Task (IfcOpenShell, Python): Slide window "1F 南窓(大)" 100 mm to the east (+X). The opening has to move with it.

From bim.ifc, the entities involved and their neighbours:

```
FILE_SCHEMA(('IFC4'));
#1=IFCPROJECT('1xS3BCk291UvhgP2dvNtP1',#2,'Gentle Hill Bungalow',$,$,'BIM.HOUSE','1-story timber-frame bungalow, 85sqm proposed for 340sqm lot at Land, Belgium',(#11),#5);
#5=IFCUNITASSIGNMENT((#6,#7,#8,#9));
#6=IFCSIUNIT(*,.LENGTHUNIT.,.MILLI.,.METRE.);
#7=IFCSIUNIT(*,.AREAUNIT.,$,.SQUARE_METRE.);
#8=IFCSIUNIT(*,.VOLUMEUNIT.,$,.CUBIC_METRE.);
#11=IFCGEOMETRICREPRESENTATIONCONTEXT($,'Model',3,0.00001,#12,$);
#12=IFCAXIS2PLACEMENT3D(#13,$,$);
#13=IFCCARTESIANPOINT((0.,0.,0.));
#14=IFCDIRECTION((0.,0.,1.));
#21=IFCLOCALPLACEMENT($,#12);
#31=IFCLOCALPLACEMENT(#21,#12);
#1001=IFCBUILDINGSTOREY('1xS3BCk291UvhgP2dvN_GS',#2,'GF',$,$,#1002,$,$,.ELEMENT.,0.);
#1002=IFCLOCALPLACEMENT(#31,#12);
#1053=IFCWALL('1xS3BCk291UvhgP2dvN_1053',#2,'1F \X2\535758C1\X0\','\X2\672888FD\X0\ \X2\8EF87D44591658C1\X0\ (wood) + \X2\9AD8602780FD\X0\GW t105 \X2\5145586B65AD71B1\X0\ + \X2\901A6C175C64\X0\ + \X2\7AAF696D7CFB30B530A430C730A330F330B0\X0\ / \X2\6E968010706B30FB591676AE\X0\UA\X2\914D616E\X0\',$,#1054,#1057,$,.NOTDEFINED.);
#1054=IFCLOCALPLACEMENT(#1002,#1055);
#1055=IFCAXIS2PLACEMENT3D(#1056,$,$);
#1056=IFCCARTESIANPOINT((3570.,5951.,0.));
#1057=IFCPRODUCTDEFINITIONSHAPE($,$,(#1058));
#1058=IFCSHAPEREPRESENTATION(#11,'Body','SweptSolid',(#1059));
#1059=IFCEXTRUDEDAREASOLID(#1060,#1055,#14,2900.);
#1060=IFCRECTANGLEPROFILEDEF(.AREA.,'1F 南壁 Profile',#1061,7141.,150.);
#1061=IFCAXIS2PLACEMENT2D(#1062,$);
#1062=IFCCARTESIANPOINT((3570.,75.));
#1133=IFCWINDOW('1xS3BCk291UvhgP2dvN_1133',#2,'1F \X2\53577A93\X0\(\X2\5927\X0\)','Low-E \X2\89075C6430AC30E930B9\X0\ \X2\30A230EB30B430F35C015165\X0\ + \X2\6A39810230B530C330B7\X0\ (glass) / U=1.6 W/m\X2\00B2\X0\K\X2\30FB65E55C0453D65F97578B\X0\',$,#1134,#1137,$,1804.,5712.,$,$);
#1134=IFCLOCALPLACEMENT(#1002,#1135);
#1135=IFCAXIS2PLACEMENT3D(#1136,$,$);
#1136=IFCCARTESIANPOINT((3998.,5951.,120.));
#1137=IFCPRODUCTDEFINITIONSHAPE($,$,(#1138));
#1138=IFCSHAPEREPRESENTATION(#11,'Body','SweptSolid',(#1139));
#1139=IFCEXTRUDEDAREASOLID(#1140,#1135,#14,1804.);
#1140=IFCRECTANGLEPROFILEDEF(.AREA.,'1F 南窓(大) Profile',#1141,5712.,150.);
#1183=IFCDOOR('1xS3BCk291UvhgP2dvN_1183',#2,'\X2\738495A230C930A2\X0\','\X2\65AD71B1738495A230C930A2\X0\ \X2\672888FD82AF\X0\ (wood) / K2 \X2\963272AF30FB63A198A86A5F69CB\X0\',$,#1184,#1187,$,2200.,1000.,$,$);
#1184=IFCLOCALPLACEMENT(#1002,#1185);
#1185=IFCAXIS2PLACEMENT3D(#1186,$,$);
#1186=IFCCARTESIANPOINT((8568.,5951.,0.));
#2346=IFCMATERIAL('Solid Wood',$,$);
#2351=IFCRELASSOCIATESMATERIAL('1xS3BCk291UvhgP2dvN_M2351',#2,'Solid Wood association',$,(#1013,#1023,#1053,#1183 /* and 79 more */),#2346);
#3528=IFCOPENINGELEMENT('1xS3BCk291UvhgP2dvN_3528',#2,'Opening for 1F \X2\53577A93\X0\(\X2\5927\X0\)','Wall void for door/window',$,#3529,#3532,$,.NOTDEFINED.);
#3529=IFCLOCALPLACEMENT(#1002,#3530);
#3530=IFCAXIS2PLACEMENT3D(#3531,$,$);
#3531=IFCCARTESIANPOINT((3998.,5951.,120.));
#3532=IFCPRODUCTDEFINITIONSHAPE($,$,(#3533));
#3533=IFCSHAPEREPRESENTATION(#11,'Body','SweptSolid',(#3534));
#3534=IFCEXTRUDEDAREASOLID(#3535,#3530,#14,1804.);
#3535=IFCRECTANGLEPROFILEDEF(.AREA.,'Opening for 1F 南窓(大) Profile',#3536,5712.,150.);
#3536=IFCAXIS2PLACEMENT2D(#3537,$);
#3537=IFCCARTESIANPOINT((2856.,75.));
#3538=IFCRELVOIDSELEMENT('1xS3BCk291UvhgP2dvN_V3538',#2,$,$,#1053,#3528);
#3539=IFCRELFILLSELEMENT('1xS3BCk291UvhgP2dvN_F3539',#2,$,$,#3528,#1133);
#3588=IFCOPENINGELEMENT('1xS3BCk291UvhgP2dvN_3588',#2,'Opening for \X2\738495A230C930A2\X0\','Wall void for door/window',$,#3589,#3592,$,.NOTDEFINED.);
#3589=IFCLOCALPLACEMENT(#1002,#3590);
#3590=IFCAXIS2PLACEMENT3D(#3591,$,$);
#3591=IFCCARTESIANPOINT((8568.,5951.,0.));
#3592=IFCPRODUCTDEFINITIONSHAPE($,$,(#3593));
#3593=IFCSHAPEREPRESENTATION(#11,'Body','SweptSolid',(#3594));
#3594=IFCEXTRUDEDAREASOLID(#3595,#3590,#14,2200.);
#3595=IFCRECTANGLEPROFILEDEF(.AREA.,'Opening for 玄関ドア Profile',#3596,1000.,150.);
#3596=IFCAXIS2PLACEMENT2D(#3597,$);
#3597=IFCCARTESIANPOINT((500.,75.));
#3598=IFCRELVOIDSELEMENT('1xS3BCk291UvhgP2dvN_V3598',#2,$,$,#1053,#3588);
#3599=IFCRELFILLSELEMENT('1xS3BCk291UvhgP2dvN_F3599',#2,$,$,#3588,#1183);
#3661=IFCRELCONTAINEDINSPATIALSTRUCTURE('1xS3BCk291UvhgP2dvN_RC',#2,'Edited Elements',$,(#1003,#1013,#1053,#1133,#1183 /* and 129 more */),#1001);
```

```python
import ifcopenshell
import ifcopenshell.api.geometry
import ifcopenshell.util.placement

model = ifcopenshell.open("bim.ifc")

window = model.by_id(1133)
opening = window.FillsVoids[0].RelatingOpeningElement
wall = opening.VoidsElements[0].RelatingBuildingElement

wall_matrix = ifcopenshell.util.placement.get_local_placement(wall.ObjectPlacement)
shift = wall_matrix[:3, 0] * 100.0
before = ifcopenshell.util.placement.get_local_placement(window.ObjectPlacement)[:3, 3].copy()

# The window is not placed relative to its opening, so move both.
for product in (opening, window):
    matrix = ifcopenshell.util.placement.get_local_placement(product.ObjectPlacement)
    matrix[:3, 3] += shift
    ifcopenshell.api.geometry.edit_object_placement(model, product=product, matrix=matrix, is_si=False)

after = ifcopenshell.util.placement.get_local_placement(window.ObjectPlacement)[:3, 3]
print("window moved by", (after - before).round(3) + 0.0)

model.write("bim_edited.ifc")
```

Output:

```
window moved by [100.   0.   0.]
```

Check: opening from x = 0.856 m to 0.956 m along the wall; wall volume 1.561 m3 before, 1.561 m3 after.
